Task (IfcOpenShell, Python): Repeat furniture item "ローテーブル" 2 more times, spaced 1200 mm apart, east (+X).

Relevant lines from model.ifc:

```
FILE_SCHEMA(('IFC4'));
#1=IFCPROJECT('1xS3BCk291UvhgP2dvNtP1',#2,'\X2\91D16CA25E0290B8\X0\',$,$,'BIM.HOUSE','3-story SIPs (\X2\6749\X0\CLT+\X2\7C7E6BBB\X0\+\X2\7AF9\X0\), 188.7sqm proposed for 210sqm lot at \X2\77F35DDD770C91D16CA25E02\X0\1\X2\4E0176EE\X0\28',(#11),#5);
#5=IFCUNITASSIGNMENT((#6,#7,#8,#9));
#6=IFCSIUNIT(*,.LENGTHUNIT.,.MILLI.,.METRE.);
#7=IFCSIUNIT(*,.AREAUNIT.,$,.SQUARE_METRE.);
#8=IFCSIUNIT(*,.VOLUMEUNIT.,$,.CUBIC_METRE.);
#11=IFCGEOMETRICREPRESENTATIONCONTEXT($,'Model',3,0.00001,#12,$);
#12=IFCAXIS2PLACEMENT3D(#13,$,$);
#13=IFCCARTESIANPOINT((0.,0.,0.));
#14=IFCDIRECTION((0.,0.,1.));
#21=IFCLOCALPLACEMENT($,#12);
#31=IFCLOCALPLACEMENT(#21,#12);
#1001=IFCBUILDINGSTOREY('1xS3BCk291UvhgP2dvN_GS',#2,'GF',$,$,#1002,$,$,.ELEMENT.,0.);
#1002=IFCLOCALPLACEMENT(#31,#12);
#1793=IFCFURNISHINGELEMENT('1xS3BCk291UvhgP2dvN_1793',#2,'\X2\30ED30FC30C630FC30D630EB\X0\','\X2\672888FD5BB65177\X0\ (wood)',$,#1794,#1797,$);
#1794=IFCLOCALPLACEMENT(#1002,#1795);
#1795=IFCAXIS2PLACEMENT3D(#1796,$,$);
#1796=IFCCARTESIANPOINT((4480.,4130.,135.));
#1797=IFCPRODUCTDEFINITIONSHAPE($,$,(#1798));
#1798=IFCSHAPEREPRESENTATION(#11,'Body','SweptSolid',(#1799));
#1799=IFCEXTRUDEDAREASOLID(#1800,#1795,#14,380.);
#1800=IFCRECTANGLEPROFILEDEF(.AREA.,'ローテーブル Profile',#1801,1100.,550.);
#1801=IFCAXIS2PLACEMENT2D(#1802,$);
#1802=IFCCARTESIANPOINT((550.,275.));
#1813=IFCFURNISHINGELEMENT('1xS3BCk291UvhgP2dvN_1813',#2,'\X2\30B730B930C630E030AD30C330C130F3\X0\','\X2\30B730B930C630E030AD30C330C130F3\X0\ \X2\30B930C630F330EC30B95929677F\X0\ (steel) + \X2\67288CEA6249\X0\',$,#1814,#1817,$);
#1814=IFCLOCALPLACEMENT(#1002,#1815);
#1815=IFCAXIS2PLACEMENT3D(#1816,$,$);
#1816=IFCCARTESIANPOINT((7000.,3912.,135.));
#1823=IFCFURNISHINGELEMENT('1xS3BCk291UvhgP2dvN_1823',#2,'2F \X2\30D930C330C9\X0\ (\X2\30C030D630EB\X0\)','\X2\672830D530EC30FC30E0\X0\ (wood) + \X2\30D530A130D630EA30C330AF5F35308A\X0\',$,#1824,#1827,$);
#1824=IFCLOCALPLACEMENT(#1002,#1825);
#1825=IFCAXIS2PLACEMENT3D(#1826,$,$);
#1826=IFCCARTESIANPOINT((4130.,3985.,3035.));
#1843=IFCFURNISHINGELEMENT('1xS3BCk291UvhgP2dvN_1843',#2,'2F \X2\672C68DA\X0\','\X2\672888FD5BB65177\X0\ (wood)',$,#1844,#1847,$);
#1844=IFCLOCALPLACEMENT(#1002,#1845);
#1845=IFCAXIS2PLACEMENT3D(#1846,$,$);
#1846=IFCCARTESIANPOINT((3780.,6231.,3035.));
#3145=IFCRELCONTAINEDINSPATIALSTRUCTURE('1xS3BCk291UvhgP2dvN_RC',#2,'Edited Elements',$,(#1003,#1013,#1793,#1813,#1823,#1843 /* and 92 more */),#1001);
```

```python
import numpy as np
import ifcopenshell
import ifcopenshell.api.geometry
import ifcopenshell.api.root
import ifcopenshell.util.element
import ifcopenshell.util.placement

model = ifcopenshell.open("model.ifc")


def reuse_history(source, copy):
    """copy_class also copies each property set's owner history, people and application; keep the originals."""
    for rel in copy.IsDefinedBy:
        if rel.is_a("IfcRelDefinesByProperties") and (history := rel.RelatingPropertyDefinition.OwnerHistory):
            rel.RelatingPropertyDefinition.OwnerHistory = source.OwnerHistory
            ifcopenshell.util.element.remove_deep2(model, history)


source = model.by_guid("1xS3BCk291UvhgP2dvN_1793")
base = ifcopenshell.util.placement.get_local_placement(source.ObjectPlacement)
step = np.array([1.0, 0.0, 0.0]) * 1200.0

for i in range(1, 3):
    copy = ifcopenshell.api.root.copy_class(model, product=source)
    copy.Representation = ifcopenshell.util.element.copy_deep(
        model, source.Representation, exclude=["IfcGeometricRepresentationContext", "IfcRepresentationMap"]
    )
    reuse_history(source, copy)
    matrix = base.copy()
    matrix[:3, 3] += i * step
    print("added at", matrix[:3, 3].round(3) + 0.0)
    ifcopenshell.api.geometry.edit_object_placement(model, product=copy, matrix=matrix, is_si=False)

model.write("model_v2.ifc")
```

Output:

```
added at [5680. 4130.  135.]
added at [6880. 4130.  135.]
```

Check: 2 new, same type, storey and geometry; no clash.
